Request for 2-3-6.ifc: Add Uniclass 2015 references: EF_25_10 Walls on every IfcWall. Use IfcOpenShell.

First a look at what the model holds.

```python
import ifcopenshell

model = ifcopenshell.open("2-3-6.ifc")
print(model.schema)
print("classifications:", [c.Name for c in model.by_type("IfcClassification")])
for ifc_class in ("IfcDoor", "IfcRoof", "IfcStair", "IfcWall", "IfcWindow"):
    print(ifc_class, len(model.by_type(ifc_class)))
```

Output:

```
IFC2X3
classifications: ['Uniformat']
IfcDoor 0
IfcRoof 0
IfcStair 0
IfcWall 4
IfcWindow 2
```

```python
import ifcopenshell
import ifcopenshell.api.classification

model = ifcopenshell.open("2-3-6.ifc")

# IFC2X3 requires Source and Edition and has no link from the project to the system.
system = model.create_entity("IfcClassification", Source="NBS", Edition="2015", Name="Uniclass 2015")

codes = {
    "IfcWall": ("EF_25_10", "Walls"),
}
for ifc_class, (code, name) in codes.items():
    products = model.by_type(ifc_class)
    ifcopenshell.api.classification.add_reference(
        model, products=products, classification=system, identification=code, name=name
    )
    print(code, len(products))

model.write("2-3-6_edited.ifc")
```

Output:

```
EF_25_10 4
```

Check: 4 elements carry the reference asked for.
